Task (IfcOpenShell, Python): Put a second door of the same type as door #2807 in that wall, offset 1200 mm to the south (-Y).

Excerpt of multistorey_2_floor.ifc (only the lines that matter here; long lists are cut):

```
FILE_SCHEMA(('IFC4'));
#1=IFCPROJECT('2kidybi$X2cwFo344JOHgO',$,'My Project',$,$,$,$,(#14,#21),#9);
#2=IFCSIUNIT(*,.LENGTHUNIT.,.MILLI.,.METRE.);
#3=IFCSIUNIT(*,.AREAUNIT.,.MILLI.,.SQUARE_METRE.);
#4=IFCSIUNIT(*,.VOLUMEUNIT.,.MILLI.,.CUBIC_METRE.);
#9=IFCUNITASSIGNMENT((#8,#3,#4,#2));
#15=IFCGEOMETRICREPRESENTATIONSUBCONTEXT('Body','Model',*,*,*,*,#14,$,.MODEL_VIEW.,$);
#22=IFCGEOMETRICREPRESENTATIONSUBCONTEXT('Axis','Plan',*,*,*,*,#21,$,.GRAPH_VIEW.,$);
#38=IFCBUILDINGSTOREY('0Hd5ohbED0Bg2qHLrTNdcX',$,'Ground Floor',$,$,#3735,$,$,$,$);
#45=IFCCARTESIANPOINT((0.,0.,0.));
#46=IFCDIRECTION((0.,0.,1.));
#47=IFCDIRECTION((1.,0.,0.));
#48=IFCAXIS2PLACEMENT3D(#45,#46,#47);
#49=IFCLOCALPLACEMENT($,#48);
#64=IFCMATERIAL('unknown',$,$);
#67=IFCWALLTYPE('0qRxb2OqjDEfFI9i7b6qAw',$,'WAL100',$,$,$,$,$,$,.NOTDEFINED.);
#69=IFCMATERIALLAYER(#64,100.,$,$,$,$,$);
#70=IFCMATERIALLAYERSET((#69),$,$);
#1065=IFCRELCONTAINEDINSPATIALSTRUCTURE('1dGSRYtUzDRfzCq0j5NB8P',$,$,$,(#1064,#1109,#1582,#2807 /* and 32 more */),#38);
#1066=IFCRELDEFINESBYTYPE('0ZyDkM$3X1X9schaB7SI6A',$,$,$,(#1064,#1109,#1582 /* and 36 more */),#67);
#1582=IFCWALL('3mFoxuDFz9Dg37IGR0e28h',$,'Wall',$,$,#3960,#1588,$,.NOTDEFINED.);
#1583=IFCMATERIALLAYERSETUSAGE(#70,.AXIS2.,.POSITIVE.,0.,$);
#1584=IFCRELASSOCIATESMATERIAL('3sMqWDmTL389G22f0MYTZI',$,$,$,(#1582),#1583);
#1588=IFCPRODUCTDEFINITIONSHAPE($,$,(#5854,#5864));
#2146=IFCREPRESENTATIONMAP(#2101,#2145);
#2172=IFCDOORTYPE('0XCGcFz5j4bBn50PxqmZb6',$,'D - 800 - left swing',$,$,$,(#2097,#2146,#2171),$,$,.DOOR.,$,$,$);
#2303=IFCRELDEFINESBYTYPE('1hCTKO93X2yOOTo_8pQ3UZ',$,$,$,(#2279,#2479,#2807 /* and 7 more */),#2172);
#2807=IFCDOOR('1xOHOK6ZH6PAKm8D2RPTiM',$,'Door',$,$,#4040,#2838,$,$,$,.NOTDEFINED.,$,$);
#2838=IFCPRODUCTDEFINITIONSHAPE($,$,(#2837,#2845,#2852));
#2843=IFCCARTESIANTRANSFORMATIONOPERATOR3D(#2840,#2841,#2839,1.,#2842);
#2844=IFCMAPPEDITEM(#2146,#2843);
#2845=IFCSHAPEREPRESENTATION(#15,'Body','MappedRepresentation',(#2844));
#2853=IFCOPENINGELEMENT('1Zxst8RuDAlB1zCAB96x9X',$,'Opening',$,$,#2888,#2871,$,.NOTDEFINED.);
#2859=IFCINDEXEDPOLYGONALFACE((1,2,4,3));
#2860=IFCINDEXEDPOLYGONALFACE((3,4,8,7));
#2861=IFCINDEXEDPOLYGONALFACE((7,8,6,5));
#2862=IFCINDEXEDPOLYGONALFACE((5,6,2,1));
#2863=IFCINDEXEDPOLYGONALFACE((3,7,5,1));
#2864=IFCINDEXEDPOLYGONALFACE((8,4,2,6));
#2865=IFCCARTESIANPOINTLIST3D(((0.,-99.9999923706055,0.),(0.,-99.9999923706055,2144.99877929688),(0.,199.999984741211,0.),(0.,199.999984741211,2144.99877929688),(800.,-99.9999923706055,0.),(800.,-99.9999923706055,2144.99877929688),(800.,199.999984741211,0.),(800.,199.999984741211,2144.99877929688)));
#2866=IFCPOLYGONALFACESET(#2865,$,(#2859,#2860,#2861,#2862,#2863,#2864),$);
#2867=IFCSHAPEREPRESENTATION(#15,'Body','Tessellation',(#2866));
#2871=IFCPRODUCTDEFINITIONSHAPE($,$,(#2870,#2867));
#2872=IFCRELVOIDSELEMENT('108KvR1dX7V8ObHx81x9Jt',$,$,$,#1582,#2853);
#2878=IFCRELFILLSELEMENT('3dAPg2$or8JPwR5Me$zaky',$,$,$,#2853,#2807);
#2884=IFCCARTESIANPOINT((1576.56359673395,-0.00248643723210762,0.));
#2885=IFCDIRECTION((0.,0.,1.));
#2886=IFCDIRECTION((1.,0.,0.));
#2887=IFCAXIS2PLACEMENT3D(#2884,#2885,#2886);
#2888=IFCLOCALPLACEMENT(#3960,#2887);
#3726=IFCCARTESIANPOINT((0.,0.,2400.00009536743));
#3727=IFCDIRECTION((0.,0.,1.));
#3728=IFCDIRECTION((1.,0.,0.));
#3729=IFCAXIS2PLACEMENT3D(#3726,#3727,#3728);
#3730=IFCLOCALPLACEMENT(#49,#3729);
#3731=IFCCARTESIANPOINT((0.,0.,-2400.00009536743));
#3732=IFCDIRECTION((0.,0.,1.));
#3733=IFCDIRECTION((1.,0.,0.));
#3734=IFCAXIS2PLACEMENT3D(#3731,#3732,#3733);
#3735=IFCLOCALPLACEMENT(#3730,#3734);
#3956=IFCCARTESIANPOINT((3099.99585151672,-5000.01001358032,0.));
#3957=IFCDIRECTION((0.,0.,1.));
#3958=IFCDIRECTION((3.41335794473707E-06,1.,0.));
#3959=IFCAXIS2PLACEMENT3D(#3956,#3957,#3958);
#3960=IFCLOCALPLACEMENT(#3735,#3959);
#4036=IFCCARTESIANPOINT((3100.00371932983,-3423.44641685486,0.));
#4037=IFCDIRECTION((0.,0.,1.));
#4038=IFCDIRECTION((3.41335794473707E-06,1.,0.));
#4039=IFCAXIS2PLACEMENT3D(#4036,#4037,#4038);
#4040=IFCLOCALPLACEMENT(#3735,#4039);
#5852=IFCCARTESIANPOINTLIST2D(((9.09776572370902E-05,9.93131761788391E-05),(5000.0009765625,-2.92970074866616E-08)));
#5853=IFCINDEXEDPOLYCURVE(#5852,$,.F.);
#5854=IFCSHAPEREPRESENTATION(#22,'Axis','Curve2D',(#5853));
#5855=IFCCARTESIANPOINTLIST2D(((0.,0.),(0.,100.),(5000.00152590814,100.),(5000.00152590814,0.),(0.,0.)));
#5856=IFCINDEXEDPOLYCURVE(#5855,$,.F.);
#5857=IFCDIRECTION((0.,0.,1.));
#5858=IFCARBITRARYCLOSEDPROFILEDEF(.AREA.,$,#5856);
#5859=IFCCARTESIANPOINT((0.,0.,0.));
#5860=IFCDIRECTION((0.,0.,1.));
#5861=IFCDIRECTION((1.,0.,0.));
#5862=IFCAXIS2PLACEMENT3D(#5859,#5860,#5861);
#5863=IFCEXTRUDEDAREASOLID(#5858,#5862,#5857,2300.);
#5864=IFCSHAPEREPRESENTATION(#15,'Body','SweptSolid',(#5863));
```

```python
import ifcopenshell
import ifcopenshell.api.feature
import ifcopenshell.api.geometry
import ifcopenshell.api.root
import ifcopenshell.geom
import ifcopenshell.util.element
import ifcopenshell.util.placement
import ifcopenshell.util.shape

model = ifcopenshell.open("multistorey_2_floor.ifc")
settings = ifcopenshell.geom.settings()


def volume(element):
    """Net volume in cubic metres, openings subtracted."""
    shape = ifcopenshell.geom.create_shape(settings, element)
    return ifcopenshell.util.shape.get_volume(shape.geometry)


door = model.by_id(2807)
opening = door.FillsVoids[0].RelatingOpeningElement
wall = opening.VoidsElements[0].RelatingBuildingElement
before = volume(wall)
shift = ifcopenshell.util.placement.get_local_placement(wall.ObjectPlacement)[:3, 0] * -1200.0

# copy_class copies the void relationship, type, container and properties, but no geometry.
new_opening = ifcopenshell.api.root.copy_class(model, product=opening)
new_opening.Representation = ifcopenshell.util.element.copy_deep(
    model, opening.Representation, exclude=["IfcGeometricRepresentationContext", "IfcRepresentationMap"]
)
new_door = ifcopenshell.api.root.copy_class(model, product=door)
new_door.Representation = ifcopenshell.util.element.copy_deep(
    model, door.Representation, exclude=["IfcGeometricRepresentationContext", "IfcRepresentationMap"]
)
ifcopenshell.api.feature.add_filling(model, opening=new_opening, element=new_door)

for old, new in ((opening, new_opening), (door, new_door)):
    matrix = ifcopenshell.util.placement.get_local_placement(old.ObjectPlacement)
    matrix[:3, 3] += shift
    ifcopenshell.api.geometry.edit_object_placement(model, product=new, matrix=matrix, is_si=False)

after = volume(wall)

print(f"wall volume {before:.3f} -> {after:.3f} m3")

model.write("multistorey_2_floor-out.ifc")
```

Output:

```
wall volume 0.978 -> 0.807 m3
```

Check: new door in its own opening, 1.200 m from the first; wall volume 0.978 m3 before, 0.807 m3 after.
